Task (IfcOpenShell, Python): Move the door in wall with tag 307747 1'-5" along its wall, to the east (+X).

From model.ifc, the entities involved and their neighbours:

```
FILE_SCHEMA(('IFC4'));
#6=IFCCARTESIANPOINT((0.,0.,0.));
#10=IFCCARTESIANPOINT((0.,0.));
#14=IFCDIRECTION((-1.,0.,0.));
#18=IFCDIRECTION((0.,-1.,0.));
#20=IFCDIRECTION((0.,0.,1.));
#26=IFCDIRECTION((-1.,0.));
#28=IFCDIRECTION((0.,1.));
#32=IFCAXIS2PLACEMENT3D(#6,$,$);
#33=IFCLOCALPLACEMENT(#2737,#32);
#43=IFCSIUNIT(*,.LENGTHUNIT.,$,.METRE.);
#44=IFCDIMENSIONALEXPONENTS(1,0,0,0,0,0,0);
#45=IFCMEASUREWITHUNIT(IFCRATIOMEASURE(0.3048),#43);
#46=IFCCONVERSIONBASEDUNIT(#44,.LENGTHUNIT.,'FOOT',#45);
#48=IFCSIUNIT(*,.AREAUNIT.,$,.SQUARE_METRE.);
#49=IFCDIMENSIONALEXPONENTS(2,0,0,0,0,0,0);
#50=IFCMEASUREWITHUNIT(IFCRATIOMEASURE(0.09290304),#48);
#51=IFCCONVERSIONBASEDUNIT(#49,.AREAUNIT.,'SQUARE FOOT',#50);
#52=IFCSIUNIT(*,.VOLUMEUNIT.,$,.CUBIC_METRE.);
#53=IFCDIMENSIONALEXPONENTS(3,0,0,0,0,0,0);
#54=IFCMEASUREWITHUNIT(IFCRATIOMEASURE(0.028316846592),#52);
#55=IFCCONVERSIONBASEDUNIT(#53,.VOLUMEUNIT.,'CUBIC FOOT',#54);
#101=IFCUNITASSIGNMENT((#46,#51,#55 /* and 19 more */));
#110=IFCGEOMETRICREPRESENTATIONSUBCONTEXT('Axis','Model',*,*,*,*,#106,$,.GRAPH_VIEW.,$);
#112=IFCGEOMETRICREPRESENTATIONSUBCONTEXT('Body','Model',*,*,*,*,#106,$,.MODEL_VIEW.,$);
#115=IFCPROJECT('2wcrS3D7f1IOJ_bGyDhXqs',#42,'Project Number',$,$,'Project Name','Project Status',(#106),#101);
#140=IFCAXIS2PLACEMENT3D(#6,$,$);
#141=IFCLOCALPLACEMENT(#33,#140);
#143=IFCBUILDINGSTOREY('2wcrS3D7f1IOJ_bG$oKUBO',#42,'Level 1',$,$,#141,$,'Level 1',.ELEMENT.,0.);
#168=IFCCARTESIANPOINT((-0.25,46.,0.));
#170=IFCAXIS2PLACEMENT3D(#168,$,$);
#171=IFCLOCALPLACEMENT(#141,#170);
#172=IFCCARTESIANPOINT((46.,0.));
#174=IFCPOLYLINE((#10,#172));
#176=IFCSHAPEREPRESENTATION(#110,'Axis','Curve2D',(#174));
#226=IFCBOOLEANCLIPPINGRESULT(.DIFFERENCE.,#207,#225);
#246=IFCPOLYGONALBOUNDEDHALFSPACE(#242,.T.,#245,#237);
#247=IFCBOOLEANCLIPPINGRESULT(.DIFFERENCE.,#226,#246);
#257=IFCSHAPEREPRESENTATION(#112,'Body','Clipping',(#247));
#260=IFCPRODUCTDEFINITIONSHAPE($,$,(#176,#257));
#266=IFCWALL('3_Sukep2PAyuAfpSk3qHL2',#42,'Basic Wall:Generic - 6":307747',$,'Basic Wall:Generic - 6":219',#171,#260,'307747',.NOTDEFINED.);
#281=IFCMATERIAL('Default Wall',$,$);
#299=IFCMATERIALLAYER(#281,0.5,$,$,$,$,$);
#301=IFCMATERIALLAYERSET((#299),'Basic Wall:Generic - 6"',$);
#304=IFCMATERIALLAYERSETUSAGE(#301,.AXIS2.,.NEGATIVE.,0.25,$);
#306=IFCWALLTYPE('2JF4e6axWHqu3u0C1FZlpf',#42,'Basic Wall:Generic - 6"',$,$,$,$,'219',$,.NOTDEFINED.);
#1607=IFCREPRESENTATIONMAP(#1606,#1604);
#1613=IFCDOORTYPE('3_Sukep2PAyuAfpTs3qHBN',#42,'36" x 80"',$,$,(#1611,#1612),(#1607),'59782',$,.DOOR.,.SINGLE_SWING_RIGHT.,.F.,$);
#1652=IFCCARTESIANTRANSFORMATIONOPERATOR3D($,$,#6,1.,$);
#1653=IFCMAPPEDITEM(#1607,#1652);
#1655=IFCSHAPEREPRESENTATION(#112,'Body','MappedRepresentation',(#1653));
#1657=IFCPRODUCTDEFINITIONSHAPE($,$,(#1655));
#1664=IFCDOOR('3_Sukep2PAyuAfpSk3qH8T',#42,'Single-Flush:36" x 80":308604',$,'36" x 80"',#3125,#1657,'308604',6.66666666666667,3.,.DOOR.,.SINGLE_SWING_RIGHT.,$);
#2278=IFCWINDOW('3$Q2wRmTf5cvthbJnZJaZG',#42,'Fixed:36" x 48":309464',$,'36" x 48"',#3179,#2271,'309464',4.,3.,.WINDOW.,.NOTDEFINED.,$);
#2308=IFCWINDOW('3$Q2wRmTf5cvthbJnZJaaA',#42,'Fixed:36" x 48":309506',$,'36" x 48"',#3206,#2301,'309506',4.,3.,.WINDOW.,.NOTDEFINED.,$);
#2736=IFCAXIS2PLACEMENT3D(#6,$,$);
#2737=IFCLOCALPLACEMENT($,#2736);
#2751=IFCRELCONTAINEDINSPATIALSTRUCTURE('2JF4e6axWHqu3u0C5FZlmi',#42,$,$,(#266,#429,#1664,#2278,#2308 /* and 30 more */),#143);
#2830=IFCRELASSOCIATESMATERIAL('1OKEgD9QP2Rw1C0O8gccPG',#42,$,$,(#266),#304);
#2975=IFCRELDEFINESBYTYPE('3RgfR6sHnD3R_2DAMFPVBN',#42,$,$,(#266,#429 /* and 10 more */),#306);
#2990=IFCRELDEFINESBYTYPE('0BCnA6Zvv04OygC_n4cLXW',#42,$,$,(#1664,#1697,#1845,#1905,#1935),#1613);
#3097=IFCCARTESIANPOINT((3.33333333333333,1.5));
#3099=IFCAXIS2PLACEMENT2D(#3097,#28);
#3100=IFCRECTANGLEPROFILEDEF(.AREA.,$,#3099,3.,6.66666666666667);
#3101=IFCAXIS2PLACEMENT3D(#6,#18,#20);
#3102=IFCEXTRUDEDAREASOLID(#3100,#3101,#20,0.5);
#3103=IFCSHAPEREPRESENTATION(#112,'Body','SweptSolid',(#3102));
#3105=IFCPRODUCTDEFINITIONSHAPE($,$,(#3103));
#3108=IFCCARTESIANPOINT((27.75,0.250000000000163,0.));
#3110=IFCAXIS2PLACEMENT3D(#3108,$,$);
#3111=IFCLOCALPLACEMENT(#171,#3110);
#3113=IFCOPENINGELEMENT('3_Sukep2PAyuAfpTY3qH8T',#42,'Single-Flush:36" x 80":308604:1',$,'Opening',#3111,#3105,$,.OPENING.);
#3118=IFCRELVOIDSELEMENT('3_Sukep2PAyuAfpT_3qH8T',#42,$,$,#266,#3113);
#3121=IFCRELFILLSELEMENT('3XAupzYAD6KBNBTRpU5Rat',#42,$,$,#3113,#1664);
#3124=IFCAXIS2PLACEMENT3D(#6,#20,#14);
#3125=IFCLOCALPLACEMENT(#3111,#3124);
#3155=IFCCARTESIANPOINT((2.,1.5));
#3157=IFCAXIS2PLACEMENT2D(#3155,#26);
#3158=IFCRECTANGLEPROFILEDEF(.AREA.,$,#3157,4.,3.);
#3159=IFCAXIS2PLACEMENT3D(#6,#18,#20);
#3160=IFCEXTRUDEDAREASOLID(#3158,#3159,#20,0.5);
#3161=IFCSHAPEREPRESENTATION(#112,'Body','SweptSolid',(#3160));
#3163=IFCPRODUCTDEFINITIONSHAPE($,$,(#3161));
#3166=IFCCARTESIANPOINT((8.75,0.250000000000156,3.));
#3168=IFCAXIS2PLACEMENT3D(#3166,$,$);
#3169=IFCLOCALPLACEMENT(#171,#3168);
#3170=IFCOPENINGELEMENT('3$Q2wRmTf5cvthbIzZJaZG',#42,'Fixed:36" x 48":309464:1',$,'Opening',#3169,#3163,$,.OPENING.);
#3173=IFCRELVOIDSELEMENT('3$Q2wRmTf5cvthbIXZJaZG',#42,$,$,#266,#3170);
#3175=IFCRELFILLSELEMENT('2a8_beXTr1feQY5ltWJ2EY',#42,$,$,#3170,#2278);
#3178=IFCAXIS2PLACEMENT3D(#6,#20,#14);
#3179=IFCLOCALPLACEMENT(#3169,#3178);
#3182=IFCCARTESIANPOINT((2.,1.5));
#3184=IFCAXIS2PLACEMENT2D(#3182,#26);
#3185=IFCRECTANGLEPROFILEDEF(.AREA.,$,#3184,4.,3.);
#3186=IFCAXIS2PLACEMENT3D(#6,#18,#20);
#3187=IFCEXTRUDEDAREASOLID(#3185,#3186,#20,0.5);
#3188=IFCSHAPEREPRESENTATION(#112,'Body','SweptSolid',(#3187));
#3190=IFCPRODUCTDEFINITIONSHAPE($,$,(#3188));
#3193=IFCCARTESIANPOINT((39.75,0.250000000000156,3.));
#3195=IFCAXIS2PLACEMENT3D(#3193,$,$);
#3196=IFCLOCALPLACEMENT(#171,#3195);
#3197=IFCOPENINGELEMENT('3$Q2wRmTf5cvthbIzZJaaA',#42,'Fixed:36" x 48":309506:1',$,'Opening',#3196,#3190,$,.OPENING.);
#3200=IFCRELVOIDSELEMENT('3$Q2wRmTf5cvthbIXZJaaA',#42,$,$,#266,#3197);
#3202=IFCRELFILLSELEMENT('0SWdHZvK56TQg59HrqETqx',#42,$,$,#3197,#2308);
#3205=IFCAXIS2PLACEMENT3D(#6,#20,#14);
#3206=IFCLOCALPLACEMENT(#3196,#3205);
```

```python
import ifcopenshell
import ifcopenshell.api.geometry
import ifcopenshell.util.placement
import ifcopenshell.util.unit

model = ifcopenshell.open("model.ifc")
unit_scale = ifcopenshell.util.unit.calculate_unit_scale(model)

door = model.by_guid("3_Sukep2PAyuAfpSk3qH8T")
opening = door.FillsVoids[0].RelatingOpeningElement
wall = opening.VoidsElements[0].RelatingBuildingElement

wall_matrix = ifcopenshell.util.placement.get_local_placement(wall.ObjectPlacement)
shift = wall_matrix[:3, 0] * 17 * 0.0254 / unit_scale
before = ifcopenshell.util.placement.get_local_placement(door.ObjectPlacement)[:3, 3].copy()

# The door is placed relative to its opening, so it follows when the opening moves.
matrix = ifcopenshell.util.placement.get_local_placement(opening.ObjectPlacement)
matrix[:3, 3] += shift
ifcopenshell.api.geometry.edit_object_placement(
    model, product=opening, matrix=matrix, is_si=False, should_transform_children=True
)

after = ifcopenshell.util.placement.get_local_placement(door.ObjectPlacement)[:3, 3]
print("door moved by", (after - before).round(3) + 0.0)

model.write("model-out.ifc")
```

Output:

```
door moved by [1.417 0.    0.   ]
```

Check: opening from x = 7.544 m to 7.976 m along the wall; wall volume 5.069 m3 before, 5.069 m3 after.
